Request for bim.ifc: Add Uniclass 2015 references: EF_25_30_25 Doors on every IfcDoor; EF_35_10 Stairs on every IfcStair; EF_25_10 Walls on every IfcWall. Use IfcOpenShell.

First a look at what the model holds.

```python
import ifcopenshell

model = ifcopenshell.open("bim.ifc")
print(model.schema)
print("classifications:", [c.Name for c in model.by_type("IfcClassification")])
for ifc_class in ("IfcDoor", "IfcRoof", "IfcStair", "IfcWall", "IfcWindow"):
    print(ifc_class, len(model.by_type(ifc_class)))
```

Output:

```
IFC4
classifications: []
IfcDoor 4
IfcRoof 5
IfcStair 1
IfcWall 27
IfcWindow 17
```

```python
import ifcopenshell
import ifcopenshell.api.classification

model = ifcopenshell.open("bim.ifc")

system = ifcopenshell.api.classification.add_classification(model, classification="Uniclass 2015")

codes = {
    "IfcDoor": ("EF_25_30_25", "Doors"),
    "IfcStair": ("EF_35_10", "Stairs"),
    "IfcWall": ("EF_25_10", "Walls"),
}
for ifc_class, (code, name) in codes.items():
    products = model.by_type(ifc_class)
    ifcopenshell.api.classification.add_reference(
        model, products=products, classification=system, identification=code, name=name
    )
    print(code, len(products))

model.write("bim_rev.ifc")
```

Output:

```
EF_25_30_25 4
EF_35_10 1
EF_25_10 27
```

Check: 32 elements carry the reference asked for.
